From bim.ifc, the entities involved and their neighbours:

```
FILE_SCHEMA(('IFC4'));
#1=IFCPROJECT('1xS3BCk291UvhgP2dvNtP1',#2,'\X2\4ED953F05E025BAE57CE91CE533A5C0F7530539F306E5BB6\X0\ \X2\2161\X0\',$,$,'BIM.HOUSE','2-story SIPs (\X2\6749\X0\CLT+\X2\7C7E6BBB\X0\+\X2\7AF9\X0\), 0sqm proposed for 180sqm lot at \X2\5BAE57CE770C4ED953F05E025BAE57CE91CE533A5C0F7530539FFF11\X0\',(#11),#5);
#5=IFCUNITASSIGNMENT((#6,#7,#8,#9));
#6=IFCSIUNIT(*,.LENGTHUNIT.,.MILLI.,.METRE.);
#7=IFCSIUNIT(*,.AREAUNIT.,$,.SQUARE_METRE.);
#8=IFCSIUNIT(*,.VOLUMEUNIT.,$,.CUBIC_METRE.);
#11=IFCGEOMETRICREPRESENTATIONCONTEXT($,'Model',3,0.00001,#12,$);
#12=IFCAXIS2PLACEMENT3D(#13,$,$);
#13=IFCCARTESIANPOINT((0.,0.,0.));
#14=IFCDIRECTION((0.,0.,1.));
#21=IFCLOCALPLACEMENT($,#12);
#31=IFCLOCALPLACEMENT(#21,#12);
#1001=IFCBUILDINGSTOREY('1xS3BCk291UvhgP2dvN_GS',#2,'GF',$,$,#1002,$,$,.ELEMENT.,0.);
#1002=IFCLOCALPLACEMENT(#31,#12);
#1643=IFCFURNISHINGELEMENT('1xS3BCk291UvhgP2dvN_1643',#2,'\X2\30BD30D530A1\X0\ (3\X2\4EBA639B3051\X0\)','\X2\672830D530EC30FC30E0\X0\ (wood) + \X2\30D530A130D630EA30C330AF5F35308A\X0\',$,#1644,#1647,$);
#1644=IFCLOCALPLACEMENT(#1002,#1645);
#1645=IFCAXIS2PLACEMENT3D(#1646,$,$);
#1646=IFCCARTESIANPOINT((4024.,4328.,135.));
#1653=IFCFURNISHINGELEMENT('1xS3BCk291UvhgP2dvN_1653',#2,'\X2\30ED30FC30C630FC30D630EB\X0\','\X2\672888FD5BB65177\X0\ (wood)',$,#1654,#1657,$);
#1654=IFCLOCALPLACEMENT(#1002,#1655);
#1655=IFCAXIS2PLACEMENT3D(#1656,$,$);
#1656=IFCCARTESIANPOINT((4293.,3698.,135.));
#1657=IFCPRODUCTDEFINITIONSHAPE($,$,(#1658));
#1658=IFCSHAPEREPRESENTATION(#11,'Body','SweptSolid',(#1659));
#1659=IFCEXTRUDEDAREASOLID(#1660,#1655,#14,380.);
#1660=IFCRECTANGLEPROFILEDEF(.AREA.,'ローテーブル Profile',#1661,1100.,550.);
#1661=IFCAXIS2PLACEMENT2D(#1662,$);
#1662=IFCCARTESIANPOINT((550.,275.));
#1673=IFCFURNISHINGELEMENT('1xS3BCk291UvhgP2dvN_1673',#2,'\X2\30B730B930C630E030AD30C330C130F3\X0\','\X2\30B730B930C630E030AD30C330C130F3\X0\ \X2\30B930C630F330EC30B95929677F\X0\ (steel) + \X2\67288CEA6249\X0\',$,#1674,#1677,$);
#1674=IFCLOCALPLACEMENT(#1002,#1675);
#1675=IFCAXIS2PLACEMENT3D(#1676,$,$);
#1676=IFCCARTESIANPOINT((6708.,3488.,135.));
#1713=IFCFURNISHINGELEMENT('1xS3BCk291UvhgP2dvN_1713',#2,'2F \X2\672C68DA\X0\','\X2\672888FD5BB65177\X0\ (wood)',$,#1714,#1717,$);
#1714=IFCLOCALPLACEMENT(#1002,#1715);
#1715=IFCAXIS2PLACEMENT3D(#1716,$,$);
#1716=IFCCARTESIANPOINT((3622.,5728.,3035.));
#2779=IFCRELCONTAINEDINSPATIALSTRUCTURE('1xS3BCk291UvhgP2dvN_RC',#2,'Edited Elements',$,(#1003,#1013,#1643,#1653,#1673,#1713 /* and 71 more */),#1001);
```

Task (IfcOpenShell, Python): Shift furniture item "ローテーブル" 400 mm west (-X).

```python
import ifcopenshell
import ifcopenshell.api.geometry
import ifcopenshell.util.placement

model = ifcopenshell.open("bim.ifc")

item = model.by_guid("1xS3BCk291UvhgP2dvN_1653")
matrix = ifcopenshell.util.placement.get_local_placement(item.ObjectPlacement)
matrix[0, 3] -= 400.0
ifcopenshell.api.geometry.edit_object_placement(model, product=item, matrix=matrix, is_si=False)

print(ifcopenshell.util.placement.get_local_placement(item.ObjectPlacement).round(3) + 0.0)

model.write("bim_updated.ifc")
```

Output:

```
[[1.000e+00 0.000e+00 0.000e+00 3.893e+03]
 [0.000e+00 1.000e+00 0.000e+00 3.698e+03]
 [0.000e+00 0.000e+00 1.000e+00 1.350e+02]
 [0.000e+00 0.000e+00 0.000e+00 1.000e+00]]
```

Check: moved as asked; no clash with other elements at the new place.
